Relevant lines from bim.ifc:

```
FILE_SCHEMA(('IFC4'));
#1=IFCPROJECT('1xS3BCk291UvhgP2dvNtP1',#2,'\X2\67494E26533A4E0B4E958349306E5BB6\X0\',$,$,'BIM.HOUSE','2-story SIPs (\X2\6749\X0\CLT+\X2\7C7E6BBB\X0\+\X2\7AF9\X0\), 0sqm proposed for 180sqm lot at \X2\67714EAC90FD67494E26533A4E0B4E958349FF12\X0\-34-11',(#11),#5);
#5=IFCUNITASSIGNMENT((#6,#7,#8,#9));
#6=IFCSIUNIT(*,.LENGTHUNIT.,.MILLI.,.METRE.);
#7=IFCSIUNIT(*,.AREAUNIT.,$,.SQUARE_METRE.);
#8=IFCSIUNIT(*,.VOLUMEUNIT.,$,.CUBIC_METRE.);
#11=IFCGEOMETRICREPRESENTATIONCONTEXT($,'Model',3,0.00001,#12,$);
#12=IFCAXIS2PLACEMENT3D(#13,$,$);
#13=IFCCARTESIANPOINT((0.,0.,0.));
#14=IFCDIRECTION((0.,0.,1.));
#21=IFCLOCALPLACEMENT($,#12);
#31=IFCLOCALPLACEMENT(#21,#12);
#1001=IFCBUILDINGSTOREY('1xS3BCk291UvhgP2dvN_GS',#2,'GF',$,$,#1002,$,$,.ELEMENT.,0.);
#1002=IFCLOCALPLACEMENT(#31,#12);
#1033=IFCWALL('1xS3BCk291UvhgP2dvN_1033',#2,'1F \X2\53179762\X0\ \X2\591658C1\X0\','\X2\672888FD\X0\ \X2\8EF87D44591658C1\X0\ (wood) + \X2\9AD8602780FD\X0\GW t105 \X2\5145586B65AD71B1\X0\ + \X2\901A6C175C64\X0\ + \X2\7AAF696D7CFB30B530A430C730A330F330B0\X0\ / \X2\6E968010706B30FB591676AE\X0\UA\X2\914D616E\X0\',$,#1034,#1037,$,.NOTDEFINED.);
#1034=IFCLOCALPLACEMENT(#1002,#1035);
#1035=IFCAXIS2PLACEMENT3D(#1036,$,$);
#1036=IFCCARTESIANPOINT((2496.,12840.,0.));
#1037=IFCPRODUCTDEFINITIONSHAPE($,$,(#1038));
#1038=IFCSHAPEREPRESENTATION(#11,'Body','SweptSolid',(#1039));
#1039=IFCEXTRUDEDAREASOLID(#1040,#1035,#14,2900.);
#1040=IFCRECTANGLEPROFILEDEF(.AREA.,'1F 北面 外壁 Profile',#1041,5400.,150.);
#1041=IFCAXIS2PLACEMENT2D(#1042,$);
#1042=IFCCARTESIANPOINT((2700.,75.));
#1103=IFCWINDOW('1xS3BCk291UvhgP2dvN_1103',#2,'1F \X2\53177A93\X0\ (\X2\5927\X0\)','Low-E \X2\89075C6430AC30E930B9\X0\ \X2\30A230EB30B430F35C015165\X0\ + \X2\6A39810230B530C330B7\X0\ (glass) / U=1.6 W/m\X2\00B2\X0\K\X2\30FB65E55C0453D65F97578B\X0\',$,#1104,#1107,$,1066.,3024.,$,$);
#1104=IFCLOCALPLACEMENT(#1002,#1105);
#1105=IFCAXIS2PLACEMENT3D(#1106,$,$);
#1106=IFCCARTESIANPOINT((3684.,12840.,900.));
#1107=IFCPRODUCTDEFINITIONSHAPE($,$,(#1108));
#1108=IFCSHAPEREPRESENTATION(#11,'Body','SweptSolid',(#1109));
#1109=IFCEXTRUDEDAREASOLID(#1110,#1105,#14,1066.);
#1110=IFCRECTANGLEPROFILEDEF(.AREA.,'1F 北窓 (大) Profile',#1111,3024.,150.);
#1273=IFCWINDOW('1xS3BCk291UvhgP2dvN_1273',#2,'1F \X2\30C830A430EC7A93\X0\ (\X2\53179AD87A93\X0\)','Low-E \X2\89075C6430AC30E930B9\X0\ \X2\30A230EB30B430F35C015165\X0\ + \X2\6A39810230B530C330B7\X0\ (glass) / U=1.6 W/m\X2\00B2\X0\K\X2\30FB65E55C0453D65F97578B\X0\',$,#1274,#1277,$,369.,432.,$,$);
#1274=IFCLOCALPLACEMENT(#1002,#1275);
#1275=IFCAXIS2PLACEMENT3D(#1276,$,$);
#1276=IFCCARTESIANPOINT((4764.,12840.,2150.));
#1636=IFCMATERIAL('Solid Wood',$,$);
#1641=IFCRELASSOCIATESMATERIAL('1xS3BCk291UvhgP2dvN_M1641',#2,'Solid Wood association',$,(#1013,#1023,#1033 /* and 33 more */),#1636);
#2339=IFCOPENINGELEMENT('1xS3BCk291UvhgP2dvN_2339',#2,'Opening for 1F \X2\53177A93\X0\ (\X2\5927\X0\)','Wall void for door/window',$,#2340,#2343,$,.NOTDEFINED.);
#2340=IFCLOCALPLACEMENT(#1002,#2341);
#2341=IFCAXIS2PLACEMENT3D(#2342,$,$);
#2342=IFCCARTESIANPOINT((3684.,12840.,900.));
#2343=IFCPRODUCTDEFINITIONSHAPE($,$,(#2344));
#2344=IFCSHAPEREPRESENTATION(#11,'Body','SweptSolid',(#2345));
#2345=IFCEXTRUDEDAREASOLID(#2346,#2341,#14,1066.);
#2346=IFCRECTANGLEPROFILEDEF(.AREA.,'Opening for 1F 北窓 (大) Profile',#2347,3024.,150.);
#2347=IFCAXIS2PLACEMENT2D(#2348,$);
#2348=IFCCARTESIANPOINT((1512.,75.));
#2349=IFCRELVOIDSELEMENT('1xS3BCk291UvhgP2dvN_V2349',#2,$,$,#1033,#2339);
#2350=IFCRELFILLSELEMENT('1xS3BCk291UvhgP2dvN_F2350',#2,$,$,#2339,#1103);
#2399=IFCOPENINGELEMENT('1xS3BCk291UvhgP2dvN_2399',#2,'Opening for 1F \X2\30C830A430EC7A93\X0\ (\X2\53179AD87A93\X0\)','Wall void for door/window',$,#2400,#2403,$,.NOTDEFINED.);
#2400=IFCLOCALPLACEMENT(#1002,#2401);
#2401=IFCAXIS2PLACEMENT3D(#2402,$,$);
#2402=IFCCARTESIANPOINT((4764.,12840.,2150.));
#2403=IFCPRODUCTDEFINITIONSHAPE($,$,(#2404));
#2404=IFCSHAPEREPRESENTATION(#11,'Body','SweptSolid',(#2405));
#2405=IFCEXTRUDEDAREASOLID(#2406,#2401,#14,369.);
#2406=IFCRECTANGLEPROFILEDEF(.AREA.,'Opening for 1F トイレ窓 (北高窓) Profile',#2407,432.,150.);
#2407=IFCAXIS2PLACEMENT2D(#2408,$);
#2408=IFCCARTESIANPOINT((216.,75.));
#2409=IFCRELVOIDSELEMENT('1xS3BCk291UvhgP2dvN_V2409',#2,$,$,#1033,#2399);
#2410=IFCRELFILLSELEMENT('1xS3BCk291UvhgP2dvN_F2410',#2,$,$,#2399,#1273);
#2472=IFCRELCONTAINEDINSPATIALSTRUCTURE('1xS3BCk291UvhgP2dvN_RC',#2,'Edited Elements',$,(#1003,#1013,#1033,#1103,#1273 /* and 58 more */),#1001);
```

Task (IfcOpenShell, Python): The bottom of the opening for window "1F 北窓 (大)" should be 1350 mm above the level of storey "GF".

```python
import numpy as np
import ifcopenshell
import ifcopenshell.api.geometry
import ifcopenshell.geom
import ifcopenshell.util.element
import ifcopenshell.util.placement
import ifcopenshell.util.shape
import ifcopenshell.util.unit

model = ifcopenshell.open("bim.ifc")
unit_scale = ifcopenshell.util.unit.calculate_unit_scale(model)

window = model.by_id(1103)
opening = window.FillsVoids[0].RelatingOpeningElement
storey = ifcopenshell.util.element.get_container(window, ifc_class="IfcBuildingStorey")
level = ifcopenshell.util.placement.get_local_placement(storey.ObjectPlacement)[2, 3]

# The opening's origin need not be at the sill, so measure its lowest point.
shape = ifcopenshell.geom.create_shape(ifcopenshell.geom.settings(), opening)
bottom = ifcopenshell.util.shape.get_shape_bottom_elevation(shape, shape.geometry) / unit_scale
dz = level + 1.35 / unit_scale - bottom

shift = np.array([0.0, 0.0, dz])
# The window is not placed relative to its opening, so move both.
for product in (opening, window):
    matrix = ifcopenshell.util.placement.get_local_placement(product.ObjectPlacement)
    matrix[:3, 3] += shift
    ifcopenshell.api.geometry.edit_object_placement(model, product=product, matrix=matrix, is_si=False)

print(f"moved by {dz * unit_scale:+.3f} m")

model.write("bim_rev.ifc")
```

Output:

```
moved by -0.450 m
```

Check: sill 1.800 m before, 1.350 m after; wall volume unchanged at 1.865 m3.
